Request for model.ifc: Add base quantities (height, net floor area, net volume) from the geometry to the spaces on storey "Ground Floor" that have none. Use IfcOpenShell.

First a look at what the model holds.

```python
import ifcopenshell
import ifcopenshell.util.element
import ifcopenshell.util.unit

model = ifcopenshell.open("model.ifc")
print(model.schema)
for unit_type in ("LENGTHUNIT", "AREAUNIT", "VOLUMEUNIT"):
    print(unit_type, ifcopenshell.util.unit.calculate_unit_scale(model, unit_type))
storey = next(s for s in model.by_type("IfcBuildingStorey") if s.Name == "Ground Floor")
spaces = [e for e in ifcopenshell.util.element.get_decomposition(storey) if e.is_a("IfcSpace")]
for e in sorted(spaces, key=lambda e: e.id()):
    print(e.id(), e.is_a(), e.Name, list(ifcopenshell.util.element.get_psets(e, qtos_only=True)), sep=" | ")
```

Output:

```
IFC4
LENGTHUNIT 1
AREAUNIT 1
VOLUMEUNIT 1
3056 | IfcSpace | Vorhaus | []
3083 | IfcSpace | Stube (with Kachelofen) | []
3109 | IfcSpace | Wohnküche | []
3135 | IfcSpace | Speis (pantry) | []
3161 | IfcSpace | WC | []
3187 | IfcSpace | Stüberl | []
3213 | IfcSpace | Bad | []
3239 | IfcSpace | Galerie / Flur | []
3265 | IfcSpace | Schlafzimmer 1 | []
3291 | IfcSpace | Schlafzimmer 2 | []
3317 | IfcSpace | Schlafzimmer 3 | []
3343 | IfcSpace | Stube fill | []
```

```python
import ifcopenshell
import ifcopenshell.api.pset
import ifcopenshell.geom
import ifcopenshell.util.element
import ifcopenshell.util.shape
import ifcopenshell.util.unit

model = ifcopenshell.open("model.ifc")
unit_scale = ifcopenshell.util.unit.calculate_unit_scale(model)
area_scale = ifcopenshell.util.unit.calculate_unit_scale(model, "AREAUNIT")
volume_scale = ifcopenshell.util.unit.calculate_unit_scale(model, "VOLUMEUNIT")
settings = ifcopenshell.geom.settings()

storey = next(s for s in model.by_type("IfcBuildingStorey") if s.Name == "Ground Floor")
spaces = [e for e in ifcopenshell.util.element.get_decomposition(storey) if e.is_a("IfcSpace")]

for e in sorted(spaces, key=lambda e: e.id()):
    if ifcopenshell.util.element.get_psets(e, qtos_only=True, should_inherit=False):
        continue
    # Geometry comes back in metres, in the element's own axes.
    shape = ifcopenshell.geom.create_shape(settings, e)
    values = {
        "Height": ifcopenshell.util.shape.get_z(shape.geometry) / unit_scale,
        "NetFloorArea": ifcopenshell.util.shape.get_footprint_area(shape.geometry) / area_scale,
        "NetVolume": ifcopenshell.util.shape.get_volume(shape.geometry) / volume_scale,
    }
    qto = ifcopenshell.api.pset.add_qto(model, product=e, name="Qto_SpaceBaseQuantities")
    ifcopenshell.api.pset.edit_qto(model, qto=qto, properties=values)
    print(e.id(), {k: round(v, 3) for k, v in values.items()})

model.write("model_v2.ifc")
```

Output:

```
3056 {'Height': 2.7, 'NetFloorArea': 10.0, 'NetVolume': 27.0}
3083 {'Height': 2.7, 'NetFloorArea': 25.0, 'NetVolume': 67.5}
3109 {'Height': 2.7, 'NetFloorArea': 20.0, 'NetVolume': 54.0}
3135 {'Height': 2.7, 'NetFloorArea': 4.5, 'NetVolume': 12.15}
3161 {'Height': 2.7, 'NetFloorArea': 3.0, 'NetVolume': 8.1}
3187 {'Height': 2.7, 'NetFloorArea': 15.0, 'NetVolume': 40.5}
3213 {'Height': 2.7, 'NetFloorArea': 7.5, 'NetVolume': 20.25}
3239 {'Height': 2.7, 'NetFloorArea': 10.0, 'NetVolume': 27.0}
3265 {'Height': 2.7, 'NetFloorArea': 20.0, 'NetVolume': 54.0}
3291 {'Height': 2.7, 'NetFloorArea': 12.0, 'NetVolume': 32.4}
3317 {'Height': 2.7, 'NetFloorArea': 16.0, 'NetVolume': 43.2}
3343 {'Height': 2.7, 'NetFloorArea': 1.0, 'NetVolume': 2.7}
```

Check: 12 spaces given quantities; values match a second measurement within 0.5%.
